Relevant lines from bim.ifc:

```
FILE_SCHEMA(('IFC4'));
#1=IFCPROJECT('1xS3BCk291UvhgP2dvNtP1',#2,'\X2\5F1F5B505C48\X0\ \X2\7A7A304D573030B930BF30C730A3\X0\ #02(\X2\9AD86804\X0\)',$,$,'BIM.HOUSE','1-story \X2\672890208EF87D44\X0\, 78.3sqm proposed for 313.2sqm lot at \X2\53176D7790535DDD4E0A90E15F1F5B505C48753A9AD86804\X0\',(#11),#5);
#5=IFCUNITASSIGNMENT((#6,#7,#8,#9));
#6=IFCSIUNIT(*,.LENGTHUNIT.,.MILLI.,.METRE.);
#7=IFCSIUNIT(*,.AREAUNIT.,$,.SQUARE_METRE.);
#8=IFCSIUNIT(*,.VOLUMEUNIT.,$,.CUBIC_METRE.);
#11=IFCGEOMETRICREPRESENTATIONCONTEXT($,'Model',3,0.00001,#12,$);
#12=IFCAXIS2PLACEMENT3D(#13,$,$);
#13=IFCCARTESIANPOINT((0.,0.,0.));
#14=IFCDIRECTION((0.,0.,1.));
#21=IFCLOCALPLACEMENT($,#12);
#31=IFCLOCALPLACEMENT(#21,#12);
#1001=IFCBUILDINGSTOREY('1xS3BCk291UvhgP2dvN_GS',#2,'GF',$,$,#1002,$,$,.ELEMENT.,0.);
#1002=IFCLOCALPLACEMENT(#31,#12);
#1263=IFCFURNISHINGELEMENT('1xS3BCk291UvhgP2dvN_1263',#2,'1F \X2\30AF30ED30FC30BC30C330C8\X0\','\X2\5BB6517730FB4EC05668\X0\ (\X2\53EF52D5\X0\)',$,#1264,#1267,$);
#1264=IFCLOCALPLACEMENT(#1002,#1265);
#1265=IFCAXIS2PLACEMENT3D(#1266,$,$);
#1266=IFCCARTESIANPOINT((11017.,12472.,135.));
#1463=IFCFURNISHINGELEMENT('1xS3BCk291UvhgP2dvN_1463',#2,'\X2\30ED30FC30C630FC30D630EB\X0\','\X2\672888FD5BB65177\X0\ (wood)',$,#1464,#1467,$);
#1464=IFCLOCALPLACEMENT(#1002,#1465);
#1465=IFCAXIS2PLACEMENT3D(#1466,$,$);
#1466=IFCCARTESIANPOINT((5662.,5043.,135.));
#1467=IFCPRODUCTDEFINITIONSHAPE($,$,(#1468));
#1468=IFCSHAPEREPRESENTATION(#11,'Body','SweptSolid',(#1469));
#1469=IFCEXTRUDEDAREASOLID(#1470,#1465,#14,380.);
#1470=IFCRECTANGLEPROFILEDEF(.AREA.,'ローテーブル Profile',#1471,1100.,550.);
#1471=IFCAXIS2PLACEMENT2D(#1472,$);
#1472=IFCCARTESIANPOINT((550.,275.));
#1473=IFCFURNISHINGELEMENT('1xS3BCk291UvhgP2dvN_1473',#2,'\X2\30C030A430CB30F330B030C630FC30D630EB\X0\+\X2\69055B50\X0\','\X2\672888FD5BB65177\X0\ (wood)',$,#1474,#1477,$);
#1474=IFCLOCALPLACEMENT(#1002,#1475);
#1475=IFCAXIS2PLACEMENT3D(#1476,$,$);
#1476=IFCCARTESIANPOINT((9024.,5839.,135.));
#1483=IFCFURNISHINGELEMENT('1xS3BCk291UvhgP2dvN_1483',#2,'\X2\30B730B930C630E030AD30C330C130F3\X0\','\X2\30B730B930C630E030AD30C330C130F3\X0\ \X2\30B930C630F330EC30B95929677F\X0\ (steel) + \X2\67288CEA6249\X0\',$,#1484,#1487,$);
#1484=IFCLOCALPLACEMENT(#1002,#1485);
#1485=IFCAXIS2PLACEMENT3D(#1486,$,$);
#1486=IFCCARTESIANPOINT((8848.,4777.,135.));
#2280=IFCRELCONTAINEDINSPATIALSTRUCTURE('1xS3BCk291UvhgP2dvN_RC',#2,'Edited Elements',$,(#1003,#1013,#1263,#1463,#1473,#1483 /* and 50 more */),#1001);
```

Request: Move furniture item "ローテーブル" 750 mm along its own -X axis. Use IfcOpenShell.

```python
import ifcopenshell
import ifcopenshell.api.geometry
import ifcopenshell.util.placement
import ifcopenshell.util.unit

model = ifcopenshell.open("bim.ifc")
unit_scale = ifcopenshell.util.unit.calculate_unit_scale(model)

item = model.by_guid("1xS3BCk291UvhgP2dvN_1463")
matrix = ifcopenshell.util.placement.get_local_placement(item.ObjectPlacement)
matrix[:3, 3] -= matrix[:3, 0] * 0.75 / unit_scale
ifcopenshell.api.geometry.edit_object_placement(model, product=item, matrix=matrix, is_si=False)

print(ifcopenshell.util.placement.get_local_placement(item.ObjectPlacement).round(3) + 0.0)

model.write("bim_edited.ifc")
```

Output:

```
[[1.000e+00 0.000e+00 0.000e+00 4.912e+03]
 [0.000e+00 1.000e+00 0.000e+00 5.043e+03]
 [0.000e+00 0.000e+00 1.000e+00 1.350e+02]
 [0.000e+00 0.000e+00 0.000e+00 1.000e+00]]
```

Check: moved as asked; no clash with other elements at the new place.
